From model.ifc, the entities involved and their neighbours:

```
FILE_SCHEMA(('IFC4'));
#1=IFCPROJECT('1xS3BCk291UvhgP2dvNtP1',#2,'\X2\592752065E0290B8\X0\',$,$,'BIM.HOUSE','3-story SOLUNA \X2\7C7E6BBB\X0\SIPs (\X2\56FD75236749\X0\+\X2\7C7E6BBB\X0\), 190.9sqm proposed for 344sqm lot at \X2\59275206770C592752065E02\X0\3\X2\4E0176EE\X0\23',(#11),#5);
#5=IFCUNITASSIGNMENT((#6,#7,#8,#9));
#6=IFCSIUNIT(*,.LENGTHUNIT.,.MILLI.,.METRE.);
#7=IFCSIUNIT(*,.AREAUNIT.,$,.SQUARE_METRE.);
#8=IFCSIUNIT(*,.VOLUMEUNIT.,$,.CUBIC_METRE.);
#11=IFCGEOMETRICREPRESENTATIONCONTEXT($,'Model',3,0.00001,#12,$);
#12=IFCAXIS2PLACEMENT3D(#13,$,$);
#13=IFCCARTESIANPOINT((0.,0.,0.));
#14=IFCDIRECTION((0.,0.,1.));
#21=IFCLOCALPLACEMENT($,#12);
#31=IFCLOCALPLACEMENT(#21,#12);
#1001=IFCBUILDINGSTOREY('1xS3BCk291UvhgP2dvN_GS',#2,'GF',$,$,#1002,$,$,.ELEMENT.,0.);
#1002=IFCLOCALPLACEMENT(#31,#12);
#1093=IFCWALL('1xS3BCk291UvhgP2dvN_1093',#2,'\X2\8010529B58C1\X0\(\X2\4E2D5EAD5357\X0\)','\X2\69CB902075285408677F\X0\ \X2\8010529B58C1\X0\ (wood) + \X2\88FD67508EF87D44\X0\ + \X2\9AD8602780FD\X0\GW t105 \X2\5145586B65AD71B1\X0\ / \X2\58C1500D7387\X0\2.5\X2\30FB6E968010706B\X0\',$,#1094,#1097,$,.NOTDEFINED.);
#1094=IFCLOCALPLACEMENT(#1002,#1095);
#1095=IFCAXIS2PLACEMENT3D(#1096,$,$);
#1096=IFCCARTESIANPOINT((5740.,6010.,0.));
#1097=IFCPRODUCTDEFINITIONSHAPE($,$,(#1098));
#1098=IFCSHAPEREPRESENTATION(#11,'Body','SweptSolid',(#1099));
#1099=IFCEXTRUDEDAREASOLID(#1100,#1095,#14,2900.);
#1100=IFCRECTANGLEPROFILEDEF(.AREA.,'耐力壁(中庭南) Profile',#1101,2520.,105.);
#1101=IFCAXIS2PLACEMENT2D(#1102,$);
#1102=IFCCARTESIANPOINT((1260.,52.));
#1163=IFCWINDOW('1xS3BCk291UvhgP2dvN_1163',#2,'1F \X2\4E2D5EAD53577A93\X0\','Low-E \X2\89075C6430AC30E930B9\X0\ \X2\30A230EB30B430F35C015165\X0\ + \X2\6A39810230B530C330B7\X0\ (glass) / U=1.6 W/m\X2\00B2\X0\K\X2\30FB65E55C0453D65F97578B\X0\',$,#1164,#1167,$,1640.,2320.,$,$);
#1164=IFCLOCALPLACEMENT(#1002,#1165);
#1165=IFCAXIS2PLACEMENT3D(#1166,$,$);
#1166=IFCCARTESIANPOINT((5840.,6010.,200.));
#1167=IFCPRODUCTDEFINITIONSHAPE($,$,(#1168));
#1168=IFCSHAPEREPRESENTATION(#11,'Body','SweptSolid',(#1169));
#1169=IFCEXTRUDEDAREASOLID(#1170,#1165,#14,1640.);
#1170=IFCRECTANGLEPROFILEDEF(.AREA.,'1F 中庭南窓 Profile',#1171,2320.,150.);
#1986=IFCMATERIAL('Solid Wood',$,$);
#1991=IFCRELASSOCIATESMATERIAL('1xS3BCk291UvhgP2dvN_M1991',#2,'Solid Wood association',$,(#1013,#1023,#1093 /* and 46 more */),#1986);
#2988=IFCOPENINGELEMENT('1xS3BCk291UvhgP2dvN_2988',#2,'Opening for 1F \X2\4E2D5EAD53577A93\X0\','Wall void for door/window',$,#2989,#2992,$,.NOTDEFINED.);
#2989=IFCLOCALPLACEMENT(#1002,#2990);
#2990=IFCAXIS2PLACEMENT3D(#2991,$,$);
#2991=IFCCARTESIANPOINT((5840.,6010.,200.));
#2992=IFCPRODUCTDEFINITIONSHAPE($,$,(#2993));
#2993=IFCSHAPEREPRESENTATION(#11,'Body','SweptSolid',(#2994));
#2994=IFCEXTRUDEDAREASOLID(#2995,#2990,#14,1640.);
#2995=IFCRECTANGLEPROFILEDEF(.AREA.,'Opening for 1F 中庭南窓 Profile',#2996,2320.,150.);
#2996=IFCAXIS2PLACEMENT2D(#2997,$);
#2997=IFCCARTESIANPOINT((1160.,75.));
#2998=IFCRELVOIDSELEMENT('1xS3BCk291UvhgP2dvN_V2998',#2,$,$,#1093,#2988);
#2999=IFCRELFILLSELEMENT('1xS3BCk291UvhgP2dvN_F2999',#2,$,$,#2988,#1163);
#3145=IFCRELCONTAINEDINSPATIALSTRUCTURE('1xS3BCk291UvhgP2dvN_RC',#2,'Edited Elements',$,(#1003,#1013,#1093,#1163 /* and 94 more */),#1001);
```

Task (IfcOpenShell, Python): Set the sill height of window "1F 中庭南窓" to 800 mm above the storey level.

```python
import numpy as np
import ifcopenshell
import ifcopenshell.api.geometry
import ifcopenshell.geom
import ifcopenshell.util.element
import ifcopenshell.util.placement
import ifcopenshell.util.shape
import ifcopenshell.util.unit

model = ifcopenshell.open("model.ifc")
unit_scale = ifcopenshell.util.unit.calculate_unit_scale(model)

window = model.by_id(1163)
opening = window.FillsVoids[0].RelatingOpeningElement
storey = ifcopenshell.util.element.get_container(window, ifc_class="IfcBuildingStorey")
level = ifcopenshell.util.placement.get_local_placement(storey.ObjectPlacement)[2, 3]

# The opening's origin need not be at the sill, so measure its lowest point.
shape = ifcopenshell.geom.create_shape(ifcopenshell.geom.settings(), opening)
bottom = ifcopenshell.util.shape.get_shape_bottom_elevation(shape, shape.geometry) / unit_scale
dz = level + 0.8 / unit_scale - bottom

shift = np.array([0.0, 0.0, dz])
# The window is not placed relative to its opening, so move both.
for product in (opening, window):
    matrix = ifcopenshell.util.placement.get_local_placement(product.ObjectPlacement)
    matrix[:3, 3] += shift
    ifcopenshell.api.geometry.edit_object_placement(model, product=product, matrix=matrix, is_si=False)

print(f"moved by {dz * unit_scale:+.3f} m")

model.write("model_v2.ifc")
```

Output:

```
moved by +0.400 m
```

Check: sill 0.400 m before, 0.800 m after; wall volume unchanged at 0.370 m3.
